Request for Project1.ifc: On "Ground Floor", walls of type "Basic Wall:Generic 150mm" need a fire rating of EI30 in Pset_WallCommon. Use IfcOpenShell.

First a look at what the model holds.

```python
import ifcopenshell
import ifcopenshell.util.element

model = ifcopenshell.open("Project1.ifc")
print(model.schema)
storey = next(s for s in model.by_type("IfcBuildingStorey") if s.Name == "Ground Floor")
walls = [e for e in ifcopenshell.util.element.get_decomposition(storey) if e.is_a("IfcWall")]
seen = {}
for e in walls:
    element_type = ifcopenshell.util.element.get_type(e)
    key = (element_type.Name if element_type != e and element_type else None, ifcopenshell.util.element.get_pset(e, "Pset_WallCommon", "FireRating"))
    seen[key] = seen.get(key, 0) + 1
for (name, value), count in sorted(seen.items(), key=str):
    print(count, "x", name, "|", value)
```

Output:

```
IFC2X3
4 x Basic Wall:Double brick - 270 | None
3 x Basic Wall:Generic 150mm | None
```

```python
import ifcopenshell
import ifcopenshell.api.pset
import ifcopenshell.util.element

model = ifcopenshell.open("Project1.ifc")

storey = next(s for s in model.by_type("IfcBuildingStorey") if s.Name == "Ground Floor")
walls = [e for e in ifcopenshell.util.element.get_decomposition(storey) if e.is_a("IfcWall")]

count = 0
for e in walls:
    element_type = ifcopenshell.util.element.get_type(e)
    if element_type in (None, e) or element_type.Name != "Basic Wall:Generic 150mm":
        continue
    # add_pset returns the element's existing set when there is one.
    pset = ifcopenshell.api.pset.add_pset(model, product=e, name="Pset_WallCommon")
    ifcopenshell.api.pset.edit_pset(model, pset=pset, properties={"FireRating": "EI30"})
    count += 1

print(count, "walls updated")

model.write("Project1_v2.ifc")
```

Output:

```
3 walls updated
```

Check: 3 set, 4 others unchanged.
